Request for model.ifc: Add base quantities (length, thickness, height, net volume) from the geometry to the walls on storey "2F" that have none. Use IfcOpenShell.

First a look at what the model holds.

```python
import ifcopenshell
import ifcopenshell.util.element
import ifcopenshell.util.unit

model = ifcopenshell.open("model.ifc")
print(model.schema)
for unit_type in ("LENGTHUNIT", "AREAUNIT", "VOLUMEUNIT"):
    print(unit_type, ifcopenshell.util.unit.calculate_unit_scale(model, unit_type))
storey = next(s for s in model.by_type("IfcBuildingStorey") if s.Name == "2F")
walls = [e for e in ifcopenshell.util.element.get_decomposition(storey) if e.is_a("IfcWall")]
for e in sorted(walls, key=lambda e: e.id()):
    print(e.id(), e.is_a(), e.Name, list(ifcopenshell.util.element.get_psets(e, qtos_only=True)), sep=" | ")
```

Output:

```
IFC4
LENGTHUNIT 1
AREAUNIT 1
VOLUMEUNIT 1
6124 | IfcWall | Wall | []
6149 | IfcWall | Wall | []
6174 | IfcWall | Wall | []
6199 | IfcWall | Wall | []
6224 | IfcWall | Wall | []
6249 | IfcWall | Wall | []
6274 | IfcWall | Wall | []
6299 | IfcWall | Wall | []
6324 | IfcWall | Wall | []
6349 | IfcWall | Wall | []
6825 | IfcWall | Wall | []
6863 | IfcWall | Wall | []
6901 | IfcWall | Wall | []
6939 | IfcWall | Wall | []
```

```python
import ifcopenshell
import ifcopenshell.api.pset
import ifcopenshell.geom
import ifcopenshell.util.element
import ifcopenshell.util.shape
import ifcopenshell.util.unit

model = ifcopenshell.open("model.ifc")
unit_scale = ifcopenshell.util.unit.calculate_unit_scale(model)
volume_scale = ifcopenshell.util.unit.calculate_unit_scale(model, "VOLUMEUNIT")
settings = ifcopenshell.geom.settings()

storey = next(s for s in model.by_type("IfcBuildingStorey") if s.Name == "2F")
walls = [e for e in ifcopenshell.util.element.get_decomposition(storey) if e.is_a("IfcWall")]

for e in sorted(walls, key=lambda e: e.id()):
    if ifcopenshell.util.element.get_psets(e, qtos_only=True, should_inherit=False):
        continue
    # Geometry comes back in metres, in the element's own axes.
    shape = ifcopenshell.geom.create_shape(settings, e)
    values = {
        "Length": ifcopenshell.util.shape.get_x(shape.geometry) / unit_scale,
        "Width": ifcopenshell.util.shape.get_y(shape.geometry) / unit_scale,
        "Height": ifcopenshell.util.shape.get_z(shape.geometry) / unit_scale,
        "NetVolume": ifcopenshell.util.shape.get_volume(shape.geometry) / volume_scale,
    }
    qto = ifcopenshell.api.pset.add_qto(model, product=e, name="Qto_WallBaseQuantities")
    ifcopenshell.api.pset.edit_qto(model, qto=qto, properties=values)
    print(e.id(), {k: round(v, 3) for k, v in values.items()})

model.write("model_updated.ifc")
```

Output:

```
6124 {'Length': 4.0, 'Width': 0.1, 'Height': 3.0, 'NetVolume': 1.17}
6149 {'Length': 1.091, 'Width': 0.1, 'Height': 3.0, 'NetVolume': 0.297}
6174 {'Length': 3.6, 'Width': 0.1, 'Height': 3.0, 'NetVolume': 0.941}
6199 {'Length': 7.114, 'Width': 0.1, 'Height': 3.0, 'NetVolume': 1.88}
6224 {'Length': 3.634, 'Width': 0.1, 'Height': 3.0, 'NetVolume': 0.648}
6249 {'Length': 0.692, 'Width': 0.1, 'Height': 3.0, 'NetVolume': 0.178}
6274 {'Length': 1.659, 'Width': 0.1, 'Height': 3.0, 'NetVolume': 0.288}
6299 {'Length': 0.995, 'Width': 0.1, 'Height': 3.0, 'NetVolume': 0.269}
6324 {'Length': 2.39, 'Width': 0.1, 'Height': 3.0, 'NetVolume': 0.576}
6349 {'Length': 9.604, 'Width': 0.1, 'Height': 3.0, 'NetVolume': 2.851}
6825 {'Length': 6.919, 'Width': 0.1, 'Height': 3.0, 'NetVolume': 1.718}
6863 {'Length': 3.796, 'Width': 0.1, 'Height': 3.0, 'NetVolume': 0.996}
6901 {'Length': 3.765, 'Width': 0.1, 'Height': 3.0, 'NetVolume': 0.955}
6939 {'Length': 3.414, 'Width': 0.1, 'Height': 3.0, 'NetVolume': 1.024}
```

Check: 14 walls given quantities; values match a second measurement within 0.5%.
